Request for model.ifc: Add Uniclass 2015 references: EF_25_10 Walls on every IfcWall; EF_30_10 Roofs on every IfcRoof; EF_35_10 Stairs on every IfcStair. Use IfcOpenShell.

First a look at what the model holds.

```python
import ifcopenshell

model = ifcopenshell.open("model.ifc")
print(model.schema)
print("classifications:", [c.Name for c in model.by_type("IfcClassification")])
for ifc_class in ("IfcDoor", "IfcRoof", "IfcStair", "IfcWall", "IfcWindow"):
    print(ifc_class, len(model.by_type(ifc_class)))
```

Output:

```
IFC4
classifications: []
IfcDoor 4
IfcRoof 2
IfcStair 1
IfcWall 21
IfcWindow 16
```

```python
import ifcopenshell
import ifcopenshell.api.classification

model = ifcopenshell.open("model.ifc")

system = ifcopenshell.api.classification.add_classification(model, classification="Uniclass 2015")

codes = {
    "IfcWall": ("EF_25_10", "Walls"),
    "IfcRoof": ("EF_30_10", "Roofs"),
    "IfcStair": ("EF_35_10", "Stairs"),
}
for ifc_class, (code, name) in codes.items():
    products = model.by_type(ifc_class)
    ifcopenshell.api.classification.add_reference(
        model, products=products, classification=system, identification=code, name=name
    )
    print(code, len(products))

model.write("model_v2.ifc")
```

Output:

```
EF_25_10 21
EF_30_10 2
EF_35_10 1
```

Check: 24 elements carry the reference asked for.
